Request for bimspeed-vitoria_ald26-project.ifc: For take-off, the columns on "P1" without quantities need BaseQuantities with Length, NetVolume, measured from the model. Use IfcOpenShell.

First a look at what the model holds.

```python
import ifcopenshell
import ifcopenshell.util.element
import ifcopenshell.util.unit

model = ifcopenshell.open("bimspeed-vitoria_ald26-project.ifc")
print(model.schema)
for unit_type in ("LENGTHUNIT", "AREAUNIT", "VOLUMEUNIT"):
    print(unit_type, ifcopenshell.util.unit.calculate_unit_scale(model, unit_type))
storey = next(s for s in model.by_type("IfcBuildingStorey") if s.Name == "P1")
columns = [e for e in ifcopenshell.util.element.get_decomposition(storey) if e.is_a("IfcColumn")]
for e in sorted(columns, key=lambda e: e.id()):
    print(e.id(), e.is_a(), e.Name, list(ifcopenshell.util.element.get_psets(e, qtos_only=True)), sep=" | ")
```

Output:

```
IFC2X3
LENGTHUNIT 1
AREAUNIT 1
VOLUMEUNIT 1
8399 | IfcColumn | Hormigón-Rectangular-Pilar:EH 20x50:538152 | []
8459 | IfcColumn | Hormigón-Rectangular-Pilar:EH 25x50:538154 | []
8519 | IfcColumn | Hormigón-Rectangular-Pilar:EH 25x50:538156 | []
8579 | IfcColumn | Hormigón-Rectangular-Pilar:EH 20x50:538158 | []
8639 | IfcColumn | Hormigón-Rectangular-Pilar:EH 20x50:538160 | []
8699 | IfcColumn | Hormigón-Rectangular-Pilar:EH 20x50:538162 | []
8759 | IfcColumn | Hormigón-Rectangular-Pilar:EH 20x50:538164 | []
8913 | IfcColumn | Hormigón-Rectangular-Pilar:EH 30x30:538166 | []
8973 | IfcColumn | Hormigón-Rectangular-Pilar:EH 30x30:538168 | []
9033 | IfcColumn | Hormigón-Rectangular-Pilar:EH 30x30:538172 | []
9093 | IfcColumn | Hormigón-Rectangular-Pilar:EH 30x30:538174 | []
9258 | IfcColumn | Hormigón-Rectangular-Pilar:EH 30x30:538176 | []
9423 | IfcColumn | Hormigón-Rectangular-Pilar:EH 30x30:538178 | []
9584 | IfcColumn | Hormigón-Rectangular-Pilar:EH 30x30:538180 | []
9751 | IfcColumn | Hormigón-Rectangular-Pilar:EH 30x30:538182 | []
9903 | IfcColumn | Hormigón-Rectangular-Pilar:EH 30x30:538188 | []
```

```python
import ifcopenshell
import ifcopenshell.api.pset
import ifcopenshell.geom
import ifcopenshell.util.element
import ifcopenshell.util.shape
import ifcopenshell.util.unit

model = ifcopenshell.open("bimspeed-vitoria_ald26-project.ifc")
unit_scale = ifcopenshell.util.unit.calculate_unit_scale(model)
volume_scale = ifcopenshell.util.unit.calculate_unit_scale(model, "VOLUMEUNIT")
settings = ifcopenshell.geom.settings()

storey = next(s for s in model.by_type("IfcBuildingStorey") if s.Name == "P1")
columns = [e for e in ifcopenshell.util.element.get_decomposition(storey) if e.is_a("IfcColumn")]

for e in sorted(columns, key=lambda e: e.id()):
    if ifcopenshell.util.element.get_psets(e, qtos_only=True, should_inherit=False):
        continue
    # Geometry comes back in metres, in the element's own axes.
    shape = ifcopenshell.geom.create_shape(settings, e)
    values = {
        "Length": ifcopenshell.util.shape.get_z(shape.geometry) / unit_scale,
        "NetVolume": ifcopenshell.util.shape.get_volume(shape.geometry) / volume_scale,
    }
    qto = ifcopenshell.api.pset.add_qto(model, product=e, name="BaseQuantities")
    ifcopenshell.api.pset.edit_qto(model, qto=qto, properties=values)
    print(e.id(), {k: round(v, 3) for k, v in values.items()})

model.write("bimspeed-vitoria_ald26-project-out.ifc")
```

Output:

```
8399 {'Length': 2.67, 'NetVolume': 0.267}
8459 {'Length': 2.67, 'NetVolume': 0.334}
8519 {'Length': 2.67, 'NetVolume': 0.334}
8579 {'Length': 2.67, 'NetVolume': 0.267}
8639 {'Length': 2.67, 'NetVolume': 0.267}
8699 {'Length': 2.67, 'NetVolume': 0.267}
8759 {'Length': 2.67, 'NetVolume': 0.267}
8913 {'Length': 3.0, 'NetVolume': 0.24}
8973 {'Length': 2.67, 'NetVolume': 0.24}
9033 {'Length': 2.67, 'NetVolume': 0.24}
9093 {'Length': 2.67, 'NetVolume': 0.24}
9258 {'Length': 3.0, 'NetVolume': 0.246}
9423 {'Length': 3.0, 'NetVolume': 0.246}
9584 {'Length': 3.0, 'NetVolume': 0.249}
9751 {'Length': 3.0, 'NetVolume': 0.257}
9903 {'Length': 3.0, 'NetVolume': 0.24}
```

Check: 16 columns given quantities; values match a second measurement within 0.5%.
